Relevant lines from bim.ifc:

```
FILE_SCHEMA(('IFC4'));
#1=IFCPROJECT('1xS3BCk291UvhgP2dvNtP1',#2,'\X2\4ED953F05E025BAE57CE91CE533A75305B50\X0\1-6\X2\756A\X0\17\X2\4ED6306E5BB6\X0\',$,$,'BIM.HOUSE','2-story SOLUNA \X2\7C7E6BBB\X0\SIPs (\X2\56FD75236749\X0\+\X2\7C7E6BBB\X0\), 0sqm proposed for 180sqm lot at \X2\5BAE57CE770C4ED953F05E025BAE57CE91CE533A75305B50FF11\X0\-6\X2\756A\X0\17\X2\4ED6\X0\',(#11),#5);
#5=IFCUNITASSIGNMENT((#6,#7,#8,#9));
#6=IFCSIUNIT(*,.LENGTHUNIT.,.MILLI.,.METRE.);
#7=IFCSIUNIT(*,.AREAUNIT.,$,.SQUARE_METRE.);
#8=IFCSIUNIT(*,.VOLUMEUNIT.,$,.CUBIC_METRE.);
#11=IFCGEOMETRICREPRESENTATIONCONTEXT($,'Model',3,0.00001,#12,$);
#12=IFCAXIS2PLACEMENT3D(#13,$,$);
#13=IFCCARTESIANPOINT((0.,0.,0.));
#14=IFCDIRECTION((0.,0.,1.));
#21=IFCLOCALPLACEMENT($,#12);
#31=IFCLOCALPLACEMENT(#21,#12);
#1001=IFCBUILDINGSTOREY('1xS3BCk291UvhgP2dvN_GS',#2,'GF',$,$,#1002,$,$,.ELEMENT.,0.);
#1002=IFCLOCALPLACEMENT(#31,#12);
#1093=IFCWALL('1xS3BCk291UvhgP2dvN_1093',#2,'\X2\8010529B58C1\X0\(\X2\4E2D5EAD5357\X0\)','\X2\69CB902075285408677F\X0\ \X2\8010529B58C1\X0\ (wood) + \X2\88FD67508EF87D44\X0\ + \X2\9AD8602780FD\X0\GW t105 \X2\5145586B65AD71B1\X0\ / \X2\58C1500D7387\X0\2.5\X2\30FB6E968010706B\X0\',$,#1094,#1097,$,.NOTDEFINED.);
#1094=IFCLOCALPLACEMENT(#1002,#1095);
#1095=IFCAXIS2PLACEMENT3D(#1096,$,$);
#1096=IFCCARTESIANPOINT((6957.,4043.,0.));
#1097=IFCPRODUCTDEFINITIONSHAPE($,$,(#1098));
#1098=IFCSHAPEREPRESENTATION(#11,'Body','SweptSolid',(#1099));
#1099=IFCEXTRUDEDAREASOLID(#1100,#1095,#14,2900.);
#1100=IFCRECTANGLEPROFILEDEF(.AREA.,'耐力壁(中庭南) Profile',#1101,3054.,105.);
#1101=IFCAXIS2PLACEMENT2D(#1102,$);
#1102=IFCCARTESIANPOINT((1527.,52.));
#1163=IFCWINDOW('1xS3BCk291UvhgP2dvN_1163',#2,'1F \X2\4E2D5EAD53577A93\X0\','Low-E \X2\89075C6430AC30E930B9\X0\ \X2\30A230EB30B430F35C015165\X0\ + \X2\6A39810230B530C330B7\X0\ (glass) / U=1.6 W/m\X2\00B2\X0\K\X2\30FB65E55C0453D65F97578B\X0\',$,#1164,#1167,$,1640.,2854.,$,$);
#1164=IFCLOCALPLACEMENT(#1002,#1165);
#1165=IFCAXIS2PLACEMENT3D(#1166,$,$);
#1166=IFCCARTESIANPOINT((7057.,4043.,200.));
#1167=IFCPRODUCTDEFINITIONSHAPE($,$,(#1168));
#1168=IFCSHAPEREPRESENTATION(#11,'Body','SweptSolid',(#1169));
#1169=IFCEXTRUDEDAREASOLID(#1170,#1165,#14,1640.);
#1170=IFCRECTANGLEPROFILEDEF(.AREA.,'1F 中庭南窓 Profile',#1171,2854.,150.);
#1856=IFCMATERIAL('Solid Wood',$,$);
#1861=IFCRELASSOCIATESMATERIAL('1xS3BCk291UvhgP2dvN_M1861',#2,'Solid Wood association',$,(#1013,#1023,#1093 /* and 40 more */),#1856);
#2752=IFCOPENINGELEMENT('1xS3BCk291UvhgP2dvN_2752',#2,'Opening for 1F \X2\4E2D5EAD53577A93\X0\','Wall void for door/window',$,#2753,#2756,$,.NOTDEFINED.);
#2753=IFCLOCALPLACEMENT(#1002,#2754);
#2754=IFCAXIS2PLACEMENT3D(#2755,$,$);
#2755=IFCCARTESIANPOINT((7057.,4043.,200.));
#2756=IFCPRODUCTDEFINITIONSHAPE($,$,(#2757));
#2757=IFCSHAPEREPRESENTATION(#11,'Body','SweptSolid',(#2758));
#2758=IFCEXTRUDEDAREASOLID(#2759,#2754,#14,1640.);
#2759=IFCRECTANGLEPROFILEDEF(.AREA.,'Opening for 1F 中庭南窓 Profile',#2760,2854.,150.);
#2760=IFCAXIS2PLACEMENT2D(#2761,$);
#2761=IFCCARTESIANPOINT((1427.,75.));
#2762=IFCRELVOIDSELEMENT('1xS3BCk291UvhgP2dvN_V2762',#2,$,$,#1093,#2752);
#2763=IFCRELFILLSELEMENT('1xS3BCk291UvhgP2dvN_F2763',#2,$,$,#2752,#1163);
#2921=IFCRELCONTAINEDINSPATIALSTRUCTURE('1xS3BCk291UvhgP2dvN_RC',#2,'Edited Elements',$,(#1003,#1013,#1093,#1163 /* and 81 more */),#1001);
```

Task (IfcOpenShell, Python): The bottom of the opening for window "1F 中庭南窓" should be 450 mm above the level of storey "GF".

```python
import numpy as np
import ifcopenshell
import ifcopenshell.api.geometry
import ifcopenshell.geom
import ifcopenshell.util.element
import ifcopenshell.util.placement
import ifcopenshell.util.shape
import ifcopenshell.util.unit

model = ifcopenshell.open("bim.ifc")
unit_scale = ifcopenshell.util.unit.calculate_unit_scale(model)

window = model.by_guid("1xS3BCk291UvhgP2dvN_1163")
opening = window.FillsVoids[0].RelatingOpeningElement
storey = ifcopenshell.util.element.get_container(window, ifc_class="IfcBuildingStorey")
level = ifcopenshell.util.placement.get_local_placement(storey.ObjectPlacement)[2, 3]

# The opening's origin need not be at the sill, so measure its lowest point.
shape = ifcopenshell.geom.create_shape(ifcopenshell.geom.settings(), opening)
bottom = ifcopenshell.util.shape.get_shape_bottom_elevation(shape, shape.geometry) / unit_scale
dz = level + 450.0 - bottom

shift = np.array([0.0, 0.0, dz])
# The window is not placed relative to its opening, so move both.
for product in (opening, window):
    matrix = ifcopenshell.util.placement.get_local_placement(product.ObjectPlacement)
    matrix[:3, 3] += shift
    ifcopenshell.api.geometry.edit_object_placement(model, product=product, matrix=matrix, is_si=False)

print(f"moved by {dz * unit_scale:+.3f} m")

model.write("bim_rev.ifc")
```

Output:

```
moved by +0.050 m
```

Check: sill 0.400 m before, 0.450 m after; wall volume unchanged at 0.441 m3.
